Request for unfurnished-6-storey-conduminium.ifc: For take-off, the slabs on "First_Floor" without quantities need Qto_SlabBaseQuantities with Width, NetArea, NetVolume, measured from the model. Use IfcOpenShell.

First a look at what the model holds.

```python
import ifcopenshell
import ifcopenshell.util.element
import ifcopenshell.util.unit

model = ifcopenshell.open("unfurnished-6-storey-conduminium.ifc")
print(model.schema)
for unit_type in ("LENGTHUNIT", "AREAUNIT", "VOLUMEUNIT"):
    print(unit_type, ifcopenshell.util.unit.calculate_unit_scale(model, unit_type))
storey = next(s for s in model.by_type("IfcBuildingStorey") if s.Name == "First_Floor")
slabs = [e for e in ifcopenshell.util.element.get_decomposition(storey) if e.is_a("IfcSlab")]
for e in sorted(slabs, key=lambda e: e.id()):
    print(e.id(), e.is_a(), e.Name, list(ifcopenshell.util.element.get_psets(e, qtos_only=True)), sep=" | ")
```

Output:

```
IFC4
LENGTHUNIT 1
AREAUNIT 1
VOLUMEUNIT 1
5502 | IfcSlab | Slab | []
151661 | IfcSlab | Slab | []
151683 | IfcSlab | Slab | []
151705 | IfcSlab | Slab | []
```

```python
import ifcopenshell
import ifcopenshell.api.pset
import ifcopenshell.geom
import ifcopenshell.util.element
import ifcopenshell.util.shape
import ifcopenshell.util.unit

model = ifcopenshell.open("unfurnished-6-storey-conduminium.ifc")
unit_scale = ifcopenshell.util.unit.calculate_unit_scale(model)
area_scale = ifcopenshell.util.unit.calculate_unit_scale(model, "AREAUNIT")
volume_scale = ifcopenshell.util.unit.calculate_unit_scale(model, "VOLUMEUNIT")
settings = ifcopenshell.geom.settings()

storey = next(s for s in model.by_type("IfcBuildingStorey") if s.Name == "First_Floor")
slabs = [e for e in ifcopenshell.util.element.get_decomposition(storey) if e.is_a("IfcSlab")]

for e in sorted(slabs, key=lambda e: e.id()):
    if ifcopenshell.util.element.get_psets(e, qtos_only=True, should_inherit=False):
        continue
    # Geometry comes back in metres, in the element's own axes.
    shape = ifcopenshell.geom.create_shape(settings, e)
    values = {
        "Width": ifcopenshell.util.shape.get_z(shape.geometry) / unit_scale,
        "NetArea": ifcopenshell.util.shape.get_footprint_area(shape.geometry) / area_scale,
        "NetVolume": ifcopenshell.util.shape.get_volume(shape.geometry) / volume_scale,
    }
    qto = ifcopenshell.api.pset.add_qto(model, product=e, name="Qto_SlabBaseQuantities")
    ifcopenshell.api.pset.edit_qto(model, qto=qto, properties=values)
    print(e.id(), {k: round(v, 3) for k, v in values.items()})

model.write("unfurnished-6-storey-conduminium_rev.ifc")
```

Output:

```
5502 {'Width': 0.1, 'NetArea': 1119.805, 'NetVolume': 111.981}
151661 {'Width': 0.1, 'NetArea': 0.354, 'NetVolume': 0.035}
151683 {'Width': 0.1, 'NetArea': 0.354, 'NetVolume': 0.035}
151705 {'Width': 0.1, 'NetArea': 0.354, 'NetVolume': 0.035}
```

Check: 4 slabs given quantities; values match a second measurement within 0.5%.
